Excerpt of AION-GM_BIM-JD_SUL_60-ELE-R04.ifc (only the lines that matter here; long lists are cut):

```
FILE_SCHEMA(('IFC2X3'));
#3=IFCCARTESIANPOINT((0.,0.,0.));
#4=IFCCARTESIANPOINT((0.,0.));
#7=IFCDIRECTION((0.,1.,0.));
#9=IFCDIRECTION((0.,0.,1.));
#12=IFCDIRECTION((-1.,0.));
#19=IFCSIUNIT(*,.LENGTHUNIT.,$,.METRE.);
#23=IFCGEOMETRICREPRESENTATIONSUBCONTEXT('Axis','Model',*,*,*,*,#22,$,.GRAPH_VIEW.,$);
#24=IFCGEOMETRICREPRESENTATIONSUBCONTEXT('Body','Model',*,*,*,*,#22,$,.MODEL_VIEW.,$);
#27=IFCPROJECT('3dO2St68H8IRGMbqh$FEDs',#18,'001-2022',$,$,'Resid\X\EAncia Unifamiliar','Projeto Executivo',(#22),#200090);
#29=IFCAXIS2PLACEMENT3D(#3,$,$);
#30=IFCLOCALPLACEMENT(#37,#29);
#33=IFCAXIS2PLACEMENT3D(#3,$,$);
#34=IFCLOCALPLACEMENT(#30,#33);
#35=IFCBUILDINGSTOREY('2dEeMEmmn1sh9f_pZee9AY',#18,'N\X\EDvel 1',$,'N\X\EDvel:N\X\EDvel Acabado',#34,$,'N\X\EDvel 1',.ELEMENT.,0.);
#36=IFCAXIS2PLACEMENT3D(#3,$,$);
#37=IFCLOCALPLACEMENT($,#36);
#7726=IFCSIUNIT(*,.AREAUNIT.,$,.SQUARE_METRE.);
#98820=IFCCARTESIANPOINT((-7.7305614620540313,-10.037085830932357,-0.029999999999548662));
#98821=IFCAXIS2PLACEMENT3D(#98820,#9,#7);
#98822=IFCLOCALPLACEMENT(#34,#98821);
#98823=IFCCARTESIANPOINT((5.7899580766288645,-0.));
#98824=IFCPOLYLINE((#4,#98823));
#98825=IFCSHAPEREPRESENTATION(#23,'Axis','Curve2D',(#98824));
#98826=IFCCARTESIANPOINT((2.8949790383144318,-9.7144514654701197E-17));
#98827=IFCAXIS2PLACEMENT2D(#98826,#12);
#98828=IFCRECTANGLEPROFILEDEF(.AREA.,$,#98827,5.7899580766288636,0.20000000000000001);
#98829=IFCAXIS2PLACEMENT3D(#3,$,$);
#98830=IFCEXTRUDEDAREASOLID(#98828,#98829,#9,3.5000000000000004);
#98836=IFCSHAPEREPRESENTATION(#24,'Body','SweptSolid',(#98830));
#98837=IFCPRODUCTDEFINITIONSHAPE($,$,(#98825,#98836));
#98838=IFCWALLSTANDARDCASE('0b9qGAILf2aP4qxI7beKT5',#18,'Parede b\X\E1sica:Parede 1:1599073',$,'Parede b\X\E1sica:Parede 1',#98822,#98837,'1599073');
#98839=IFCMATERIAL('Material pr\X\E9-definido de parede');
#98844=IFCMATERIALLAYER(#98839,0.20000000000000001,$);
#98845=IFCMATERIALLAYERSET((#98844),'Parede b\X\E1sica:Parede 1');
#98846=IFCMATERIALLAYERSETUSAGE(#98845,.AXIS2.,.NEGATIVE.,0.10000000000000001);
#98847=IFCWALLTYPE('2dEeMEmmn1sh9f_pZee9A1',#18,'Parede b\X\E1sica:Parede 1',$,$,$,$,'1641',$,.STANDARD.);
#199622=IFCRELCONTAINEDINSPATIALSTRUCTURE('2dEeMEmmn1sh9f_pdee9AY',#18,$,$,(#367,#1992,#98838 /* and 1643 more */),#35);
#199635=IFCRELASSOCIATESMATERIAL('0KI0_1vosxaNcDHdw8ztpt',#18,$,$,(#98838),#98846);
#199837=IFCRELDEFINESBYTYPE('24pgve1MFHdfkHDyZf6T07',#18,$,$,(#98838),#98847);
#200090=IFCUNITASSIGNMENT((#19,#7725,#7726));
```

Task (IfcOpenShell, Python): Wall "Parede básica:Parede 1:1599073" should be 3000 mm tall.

```python
import ifcopenshell
import ifcopenshell.geom
import ifcopenshell.util.representation
import ifcopenshell.util.shape
import ifcopenshell.util.unit

model = ifcopenshell.open("AION-GM_BIM-JD_SUL_60-ELE-R04.ifc")
unit_scale = ifcopenshell.util.unit.calculate_unit_scale(model)
settings = ifcopenshell.geom.settings()


def volume(element):
    """Net volume in cubic metres, openings subtracted."""
    shape = ifcopenshell.geom.create_shape(settings, element)
    return ifcopenshell.util.shape.get_volume(shape.geometry)


wall = model.by_guid("0b9qGAILf2aP4qxI7beKT5")
before = volume(wall)

body = ifcopenshell.util.representation.get_representation(wall, "Model", "Body")
solid = body.Items[0]
old_height = solid.Depth
solid.Depth = 3 / unit_scale
after = volume(wall)

print(f"height {old_height:g} -> {solid.Depth:g}, volume {before:.3f} -> {after:.3f} m3")

model.write("AION-GM_BIM-JD_SUL_60-ELE-R04_v2.ifc")
```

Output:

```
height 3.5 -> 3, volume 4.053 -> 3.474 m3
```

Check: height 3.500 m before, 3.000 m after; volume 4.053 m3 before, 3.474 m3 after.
